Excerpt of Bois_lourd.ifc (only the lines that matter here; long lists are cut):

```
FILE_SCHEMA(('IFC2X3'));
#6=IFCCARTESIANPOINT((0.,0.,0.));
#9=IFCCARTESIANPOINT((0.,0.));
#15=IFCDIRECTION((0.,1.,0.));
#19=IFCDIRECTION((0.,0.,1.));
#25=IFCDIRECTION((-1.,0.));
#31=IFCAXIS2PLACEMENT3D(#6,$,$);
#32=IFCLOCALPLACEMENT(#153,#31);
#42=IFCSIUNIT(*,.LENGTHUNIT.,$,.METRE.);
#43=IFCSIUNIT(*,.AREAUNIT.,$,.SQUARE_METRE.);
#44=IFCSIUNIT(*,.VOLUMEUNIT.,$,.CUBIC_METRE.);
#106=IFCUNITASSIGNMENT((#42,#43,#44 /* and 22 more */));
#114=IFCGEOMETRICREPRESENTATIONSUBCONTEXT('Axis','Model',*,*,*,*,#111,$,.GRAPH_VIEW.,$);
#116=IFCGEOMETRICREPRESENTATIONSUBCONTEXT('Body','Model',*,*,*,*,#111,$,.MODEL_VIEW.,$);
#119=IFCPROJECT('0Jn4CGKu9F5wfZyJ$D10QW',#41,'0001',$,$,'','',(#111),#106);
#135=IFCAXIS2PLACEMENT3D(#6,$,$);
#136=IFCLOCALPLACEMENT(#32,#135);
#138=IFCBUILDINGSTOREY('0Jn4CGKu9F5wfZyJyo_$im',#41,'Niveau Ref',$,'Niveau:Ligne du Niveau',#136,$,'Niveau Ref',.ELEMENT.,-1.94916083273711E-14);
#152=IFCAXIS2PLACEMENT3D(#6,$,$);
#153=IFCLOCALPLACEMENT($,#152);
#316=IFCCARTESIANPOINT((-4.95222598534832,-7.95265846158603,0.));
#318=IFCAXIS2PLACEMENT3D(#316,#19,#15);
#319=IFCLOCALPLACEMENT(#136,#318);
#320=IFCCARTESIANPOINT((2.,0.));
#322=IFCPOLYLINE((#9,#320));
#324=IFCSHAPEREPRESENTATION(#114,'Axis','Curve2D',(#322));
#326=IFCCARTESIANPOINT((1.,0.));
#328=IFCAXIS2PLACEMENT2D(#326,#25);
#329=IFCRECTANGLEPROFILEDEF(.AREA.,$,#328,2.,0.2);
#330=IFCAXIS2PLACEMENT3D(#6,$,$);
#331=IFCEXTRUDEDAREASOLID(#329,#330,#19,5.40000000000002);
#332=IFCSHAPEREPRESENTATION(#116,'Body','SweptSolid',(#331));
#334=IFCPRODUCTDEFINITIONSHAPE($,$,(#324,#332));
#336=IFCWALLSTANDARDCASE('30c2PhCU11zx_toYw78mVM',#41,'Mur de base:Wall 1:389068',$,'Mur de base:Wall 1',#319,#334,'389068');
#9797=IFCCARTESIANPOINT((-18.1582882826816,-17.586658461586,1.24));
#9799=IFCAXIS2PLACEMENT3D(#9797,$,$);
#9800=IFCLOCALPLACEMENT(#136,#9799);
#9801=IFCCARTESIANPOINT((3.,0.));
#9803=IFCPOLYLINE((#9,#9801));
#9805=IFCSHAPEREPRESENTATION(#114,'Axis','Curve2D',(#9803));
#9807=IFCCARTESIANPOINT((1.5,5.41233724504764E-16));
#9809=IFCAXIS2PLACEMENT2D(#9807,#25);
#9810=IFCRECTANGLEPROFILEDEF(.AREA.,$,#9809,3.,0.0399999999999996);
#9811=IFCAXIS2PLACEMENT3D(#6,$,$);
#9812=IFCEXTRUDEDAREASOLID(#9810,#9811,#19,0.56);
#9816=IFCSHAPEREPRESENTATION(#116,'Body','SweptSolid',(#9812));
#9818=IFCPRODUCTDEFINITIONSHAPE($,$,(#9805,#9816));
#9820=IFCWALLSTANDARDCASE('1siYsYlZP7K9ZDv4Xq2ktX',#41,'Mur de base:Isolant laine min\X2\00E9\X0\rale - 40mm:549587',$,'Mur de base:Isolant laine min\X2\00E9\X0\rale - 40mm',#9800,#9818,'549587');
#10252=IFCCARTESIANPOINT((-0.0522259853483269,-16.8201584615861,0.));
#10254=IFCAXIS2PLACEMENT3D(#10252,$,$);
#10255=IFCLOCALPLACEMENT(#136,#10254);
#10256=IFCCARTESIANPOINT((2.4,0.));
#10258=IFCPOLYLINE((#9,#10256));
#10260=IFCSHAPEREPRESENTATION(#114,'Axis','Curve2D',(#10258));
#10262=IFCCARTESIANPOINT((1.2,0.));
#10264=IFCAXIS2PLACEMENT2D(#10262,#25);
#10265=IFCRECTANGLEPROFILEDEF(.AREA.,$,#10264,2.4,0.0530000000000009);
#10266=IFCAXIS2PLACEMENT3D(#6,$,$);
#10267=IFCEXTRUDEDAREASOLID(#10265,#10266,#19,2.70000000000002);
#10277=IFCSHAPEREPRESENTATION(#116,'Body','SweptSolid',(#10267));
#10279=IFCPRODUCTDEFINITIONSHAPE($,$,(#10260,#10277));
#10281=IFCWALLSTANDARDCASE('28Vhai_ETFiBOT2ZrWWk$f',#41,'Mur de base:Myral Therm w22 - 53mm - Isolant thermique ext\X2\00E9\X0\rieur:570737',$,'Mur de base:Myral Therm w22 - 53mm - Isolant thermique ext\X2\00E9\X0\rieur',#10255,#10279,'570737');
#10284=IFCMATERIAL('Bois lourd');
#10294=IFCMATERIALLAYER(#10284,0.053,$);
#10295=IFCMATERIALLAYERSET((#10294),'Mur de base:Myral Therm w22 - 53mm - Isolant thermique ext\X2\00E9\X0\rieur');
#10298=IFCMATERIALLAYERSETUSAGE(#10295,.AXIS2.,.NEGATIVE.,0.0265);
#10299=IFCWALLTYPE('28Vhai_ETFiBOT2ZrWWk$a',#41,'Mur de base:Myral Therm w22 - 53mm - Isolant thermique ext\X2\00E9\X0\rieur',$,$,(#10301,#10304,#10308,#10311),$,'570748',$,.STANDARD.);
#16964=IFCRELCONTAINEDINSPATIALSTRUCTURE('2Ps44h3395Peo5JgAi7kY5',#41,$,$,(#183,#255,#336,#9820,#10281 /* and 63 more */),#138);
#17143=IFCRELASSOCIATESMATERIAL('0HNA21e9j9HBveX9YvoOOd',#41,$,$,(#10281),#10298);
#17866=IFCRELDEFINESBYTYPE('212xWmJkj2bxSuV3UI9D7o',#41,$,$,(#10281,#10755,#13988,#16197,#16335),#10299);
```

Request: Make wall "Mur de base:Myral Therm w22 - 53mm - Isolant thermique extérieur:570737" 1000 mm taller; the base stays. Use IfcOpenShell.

```python
import ifcopenshell
import ifcopenshell.geom
import ifcopenshell.util.representation
import ifcopenshell.util.shape

model = ifcopenshell.open("Bois_lourd.ifc")
settings = ifcopenshell.geom.settings()


def volume(element):
    """Net volume in cubic metres, openings subtracted."""
    shape = ifcopenshell.geom.create_shape(settings, element)
    return ifcopenshell.util.shape.get_volume(shape.geometry)


wall = model.by_guid("28Vhai_ETFiBOT2ZrWWk$f")
before = volume(wall)

body = ifcopenshell.util.representation.get_representation(wall, "Model", "Body")
solid = body.Items[0]
old_height = solid.Depth
solid.Depth += 1.0
after = volume(wall)

print(f"height {old_height:g} -> {solid.Depth:g}, volume {before:.3f} -> {after:.3f} m3")

model.write("Bois_lourd_rev.ifc")
```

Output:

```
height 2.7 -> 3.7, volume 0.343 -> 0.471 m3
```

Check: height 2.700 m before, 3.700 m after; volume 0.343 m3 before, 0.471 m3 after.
